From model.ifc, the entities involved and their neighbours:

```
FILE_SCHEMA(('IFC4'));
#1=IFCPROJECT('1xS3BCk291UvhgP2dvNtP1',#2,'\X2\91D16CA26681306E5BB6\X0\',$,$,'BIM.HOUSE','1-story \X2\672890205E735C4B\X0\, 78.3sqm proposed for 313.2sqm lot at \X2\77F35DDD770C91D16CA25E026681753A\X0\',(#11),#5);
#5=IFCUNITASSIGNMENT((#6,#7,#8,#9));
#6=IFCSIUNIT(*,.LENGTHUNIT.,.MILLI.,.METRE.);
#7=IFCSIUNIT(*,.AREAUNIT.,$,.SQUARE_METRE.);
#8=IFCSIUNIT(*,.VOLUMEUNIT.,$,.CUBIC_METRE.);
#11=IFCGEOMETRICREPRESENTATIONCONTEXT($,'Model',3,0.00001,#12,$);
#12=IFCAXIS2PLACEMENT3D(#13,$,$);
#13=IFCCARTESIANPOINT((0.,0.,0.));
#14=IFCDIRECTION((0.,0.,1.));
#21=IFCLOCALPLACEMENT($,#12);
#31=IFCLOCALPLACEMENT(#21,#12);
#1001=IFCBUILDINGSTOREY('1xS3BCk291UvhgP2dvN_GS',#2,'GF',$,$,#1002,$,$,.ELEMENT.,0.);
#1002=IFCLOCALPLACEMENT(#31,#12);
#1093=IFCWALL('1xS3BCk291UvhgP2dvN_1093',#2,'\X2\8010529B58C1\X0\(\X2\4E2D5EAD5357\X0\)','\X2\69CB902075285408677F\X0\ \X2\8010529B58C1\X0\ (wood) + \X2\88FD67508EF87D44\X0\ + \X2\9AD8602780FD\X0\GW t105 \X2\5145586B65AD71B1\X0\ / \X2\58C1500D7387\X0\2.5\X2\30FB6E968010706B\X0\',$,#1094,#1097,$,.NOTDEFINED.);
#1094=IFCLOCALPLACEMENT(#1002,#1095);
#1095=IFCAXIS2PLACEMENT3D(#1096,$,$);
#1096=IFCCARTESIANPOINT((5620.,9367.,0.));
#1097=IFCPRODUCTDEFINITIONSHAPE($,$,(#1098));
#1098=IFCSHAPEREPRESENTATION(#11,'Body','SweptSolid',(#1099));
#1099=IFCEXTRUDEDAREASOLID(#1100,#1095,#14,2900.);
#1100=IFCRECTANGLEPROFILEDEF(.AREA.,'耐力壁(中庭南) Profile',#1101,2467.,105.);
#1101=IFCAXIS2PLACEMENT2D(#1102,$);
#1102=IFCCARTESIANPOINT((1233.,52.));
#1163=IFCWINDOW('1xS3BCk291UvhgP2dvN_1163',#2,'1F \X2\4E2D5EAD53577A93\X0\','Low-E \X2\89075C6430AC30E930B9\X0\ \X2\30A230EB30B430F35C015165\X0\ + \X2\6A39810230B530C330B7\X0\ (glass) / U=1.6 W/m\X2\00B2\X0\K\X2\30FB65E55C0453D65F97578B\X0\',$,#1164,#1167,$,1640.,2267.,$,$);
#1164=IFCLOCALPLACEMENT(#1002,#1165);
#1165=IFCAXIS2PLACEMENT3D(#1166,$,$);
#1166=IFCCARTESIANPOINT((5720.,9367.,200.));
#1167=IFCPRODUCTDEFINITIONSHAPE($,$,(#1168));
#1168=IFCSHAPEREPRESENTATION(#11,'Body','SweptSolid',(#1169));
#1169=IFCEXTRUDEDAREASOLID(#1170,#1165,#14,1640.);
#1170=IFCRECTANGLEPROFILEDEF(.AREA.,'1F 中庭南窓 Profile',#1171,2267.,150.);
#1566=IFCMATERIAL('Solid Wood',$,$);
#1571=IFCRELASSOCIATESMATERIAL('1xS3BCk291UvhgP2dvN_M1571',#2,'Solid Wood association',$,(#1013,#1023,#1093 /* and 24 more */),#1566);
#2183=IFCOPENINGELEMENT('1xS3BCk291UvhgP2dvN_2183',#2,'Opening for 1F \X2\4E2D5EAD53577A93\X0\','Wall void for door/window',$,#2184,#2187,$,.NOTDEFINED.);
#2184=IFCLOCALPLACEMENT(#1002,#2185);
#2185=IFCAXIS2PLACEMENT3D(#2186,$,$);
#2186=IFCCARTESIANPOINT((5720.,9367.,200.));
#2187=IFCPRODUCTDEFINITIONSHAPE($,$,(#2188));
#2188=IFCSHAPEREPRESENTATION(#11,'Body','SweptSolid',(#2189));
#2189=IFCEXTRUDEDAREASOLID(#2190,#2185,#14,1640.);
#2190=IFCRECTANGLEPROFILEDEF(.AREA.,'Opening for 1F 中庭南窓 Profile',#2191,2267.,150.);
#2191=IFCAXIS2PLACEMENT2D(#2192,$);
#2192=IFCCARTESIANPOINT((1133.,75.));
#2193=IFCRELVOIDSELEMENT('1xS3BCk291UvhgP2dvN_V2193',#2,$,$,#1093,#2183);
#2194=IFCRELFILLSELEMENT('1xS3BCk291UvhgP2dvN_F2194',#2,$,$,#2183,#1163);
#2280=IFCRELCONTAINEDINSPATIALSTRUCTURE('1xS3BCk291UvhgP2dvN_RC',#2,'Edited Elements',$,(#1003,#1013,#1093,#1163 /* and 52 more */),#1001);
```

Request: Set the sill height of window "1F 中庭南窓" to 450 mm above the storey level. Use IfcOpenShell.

```python
import numpy as np
import ifcopenshell
import ifcopenshell.api.geometry
import ifcopenshell.geom
import ifcopenshell.util.element
import ifcopenshell.util.placement
import ifcopenshell.util.shape
import ifcopenshell.util.unit

model = ifcopenshell.open("model.ifc")
unit_scale = ifcopenshell.util.unit.calculate_unit_scale(model)

window = model.by_id(1163)
opening = window.FillsVoids[0].RelatingOpeningElement
storey = ifcopenshell.util.element.get_container(window, ifc_class="IfcBuildingStorey")
level = ifcopenshell.util.placement.get_local_placement(storey.ObjectPlacement)[2, 3]

# The opening's origin need not be at the sill, so measure its lowest point.
shape = ifcopenshell.geom.create_shape(ifcopenshell.geom.settings(), opening)
bottom = ifcopenshell.util.shape.get_shape_bottom_elevation(shape, shape.geometry) / unit_scale
dz = level + 0.45 / unit_scale - bottom

shift = np.array([0.0, 0.0, dz])
# The window is not placed relative to its opening, so move both.
for product in (opening, window):
    matrix = ifcopenshell.util.placement.get_local_placement(product.ObjectPlacement)
    matrix[:3, 3] += shift
    ifcopenshell.api.geometry.edit_object_placement(model, product=product, matrix=matrix, is_si=False)

print(f"moved by {dz * unit_scale:+.3f} m")

model.write("model_updated.ifc")
```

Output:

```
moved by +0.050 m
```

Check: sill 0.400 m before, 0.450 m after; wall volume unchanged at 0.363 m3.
